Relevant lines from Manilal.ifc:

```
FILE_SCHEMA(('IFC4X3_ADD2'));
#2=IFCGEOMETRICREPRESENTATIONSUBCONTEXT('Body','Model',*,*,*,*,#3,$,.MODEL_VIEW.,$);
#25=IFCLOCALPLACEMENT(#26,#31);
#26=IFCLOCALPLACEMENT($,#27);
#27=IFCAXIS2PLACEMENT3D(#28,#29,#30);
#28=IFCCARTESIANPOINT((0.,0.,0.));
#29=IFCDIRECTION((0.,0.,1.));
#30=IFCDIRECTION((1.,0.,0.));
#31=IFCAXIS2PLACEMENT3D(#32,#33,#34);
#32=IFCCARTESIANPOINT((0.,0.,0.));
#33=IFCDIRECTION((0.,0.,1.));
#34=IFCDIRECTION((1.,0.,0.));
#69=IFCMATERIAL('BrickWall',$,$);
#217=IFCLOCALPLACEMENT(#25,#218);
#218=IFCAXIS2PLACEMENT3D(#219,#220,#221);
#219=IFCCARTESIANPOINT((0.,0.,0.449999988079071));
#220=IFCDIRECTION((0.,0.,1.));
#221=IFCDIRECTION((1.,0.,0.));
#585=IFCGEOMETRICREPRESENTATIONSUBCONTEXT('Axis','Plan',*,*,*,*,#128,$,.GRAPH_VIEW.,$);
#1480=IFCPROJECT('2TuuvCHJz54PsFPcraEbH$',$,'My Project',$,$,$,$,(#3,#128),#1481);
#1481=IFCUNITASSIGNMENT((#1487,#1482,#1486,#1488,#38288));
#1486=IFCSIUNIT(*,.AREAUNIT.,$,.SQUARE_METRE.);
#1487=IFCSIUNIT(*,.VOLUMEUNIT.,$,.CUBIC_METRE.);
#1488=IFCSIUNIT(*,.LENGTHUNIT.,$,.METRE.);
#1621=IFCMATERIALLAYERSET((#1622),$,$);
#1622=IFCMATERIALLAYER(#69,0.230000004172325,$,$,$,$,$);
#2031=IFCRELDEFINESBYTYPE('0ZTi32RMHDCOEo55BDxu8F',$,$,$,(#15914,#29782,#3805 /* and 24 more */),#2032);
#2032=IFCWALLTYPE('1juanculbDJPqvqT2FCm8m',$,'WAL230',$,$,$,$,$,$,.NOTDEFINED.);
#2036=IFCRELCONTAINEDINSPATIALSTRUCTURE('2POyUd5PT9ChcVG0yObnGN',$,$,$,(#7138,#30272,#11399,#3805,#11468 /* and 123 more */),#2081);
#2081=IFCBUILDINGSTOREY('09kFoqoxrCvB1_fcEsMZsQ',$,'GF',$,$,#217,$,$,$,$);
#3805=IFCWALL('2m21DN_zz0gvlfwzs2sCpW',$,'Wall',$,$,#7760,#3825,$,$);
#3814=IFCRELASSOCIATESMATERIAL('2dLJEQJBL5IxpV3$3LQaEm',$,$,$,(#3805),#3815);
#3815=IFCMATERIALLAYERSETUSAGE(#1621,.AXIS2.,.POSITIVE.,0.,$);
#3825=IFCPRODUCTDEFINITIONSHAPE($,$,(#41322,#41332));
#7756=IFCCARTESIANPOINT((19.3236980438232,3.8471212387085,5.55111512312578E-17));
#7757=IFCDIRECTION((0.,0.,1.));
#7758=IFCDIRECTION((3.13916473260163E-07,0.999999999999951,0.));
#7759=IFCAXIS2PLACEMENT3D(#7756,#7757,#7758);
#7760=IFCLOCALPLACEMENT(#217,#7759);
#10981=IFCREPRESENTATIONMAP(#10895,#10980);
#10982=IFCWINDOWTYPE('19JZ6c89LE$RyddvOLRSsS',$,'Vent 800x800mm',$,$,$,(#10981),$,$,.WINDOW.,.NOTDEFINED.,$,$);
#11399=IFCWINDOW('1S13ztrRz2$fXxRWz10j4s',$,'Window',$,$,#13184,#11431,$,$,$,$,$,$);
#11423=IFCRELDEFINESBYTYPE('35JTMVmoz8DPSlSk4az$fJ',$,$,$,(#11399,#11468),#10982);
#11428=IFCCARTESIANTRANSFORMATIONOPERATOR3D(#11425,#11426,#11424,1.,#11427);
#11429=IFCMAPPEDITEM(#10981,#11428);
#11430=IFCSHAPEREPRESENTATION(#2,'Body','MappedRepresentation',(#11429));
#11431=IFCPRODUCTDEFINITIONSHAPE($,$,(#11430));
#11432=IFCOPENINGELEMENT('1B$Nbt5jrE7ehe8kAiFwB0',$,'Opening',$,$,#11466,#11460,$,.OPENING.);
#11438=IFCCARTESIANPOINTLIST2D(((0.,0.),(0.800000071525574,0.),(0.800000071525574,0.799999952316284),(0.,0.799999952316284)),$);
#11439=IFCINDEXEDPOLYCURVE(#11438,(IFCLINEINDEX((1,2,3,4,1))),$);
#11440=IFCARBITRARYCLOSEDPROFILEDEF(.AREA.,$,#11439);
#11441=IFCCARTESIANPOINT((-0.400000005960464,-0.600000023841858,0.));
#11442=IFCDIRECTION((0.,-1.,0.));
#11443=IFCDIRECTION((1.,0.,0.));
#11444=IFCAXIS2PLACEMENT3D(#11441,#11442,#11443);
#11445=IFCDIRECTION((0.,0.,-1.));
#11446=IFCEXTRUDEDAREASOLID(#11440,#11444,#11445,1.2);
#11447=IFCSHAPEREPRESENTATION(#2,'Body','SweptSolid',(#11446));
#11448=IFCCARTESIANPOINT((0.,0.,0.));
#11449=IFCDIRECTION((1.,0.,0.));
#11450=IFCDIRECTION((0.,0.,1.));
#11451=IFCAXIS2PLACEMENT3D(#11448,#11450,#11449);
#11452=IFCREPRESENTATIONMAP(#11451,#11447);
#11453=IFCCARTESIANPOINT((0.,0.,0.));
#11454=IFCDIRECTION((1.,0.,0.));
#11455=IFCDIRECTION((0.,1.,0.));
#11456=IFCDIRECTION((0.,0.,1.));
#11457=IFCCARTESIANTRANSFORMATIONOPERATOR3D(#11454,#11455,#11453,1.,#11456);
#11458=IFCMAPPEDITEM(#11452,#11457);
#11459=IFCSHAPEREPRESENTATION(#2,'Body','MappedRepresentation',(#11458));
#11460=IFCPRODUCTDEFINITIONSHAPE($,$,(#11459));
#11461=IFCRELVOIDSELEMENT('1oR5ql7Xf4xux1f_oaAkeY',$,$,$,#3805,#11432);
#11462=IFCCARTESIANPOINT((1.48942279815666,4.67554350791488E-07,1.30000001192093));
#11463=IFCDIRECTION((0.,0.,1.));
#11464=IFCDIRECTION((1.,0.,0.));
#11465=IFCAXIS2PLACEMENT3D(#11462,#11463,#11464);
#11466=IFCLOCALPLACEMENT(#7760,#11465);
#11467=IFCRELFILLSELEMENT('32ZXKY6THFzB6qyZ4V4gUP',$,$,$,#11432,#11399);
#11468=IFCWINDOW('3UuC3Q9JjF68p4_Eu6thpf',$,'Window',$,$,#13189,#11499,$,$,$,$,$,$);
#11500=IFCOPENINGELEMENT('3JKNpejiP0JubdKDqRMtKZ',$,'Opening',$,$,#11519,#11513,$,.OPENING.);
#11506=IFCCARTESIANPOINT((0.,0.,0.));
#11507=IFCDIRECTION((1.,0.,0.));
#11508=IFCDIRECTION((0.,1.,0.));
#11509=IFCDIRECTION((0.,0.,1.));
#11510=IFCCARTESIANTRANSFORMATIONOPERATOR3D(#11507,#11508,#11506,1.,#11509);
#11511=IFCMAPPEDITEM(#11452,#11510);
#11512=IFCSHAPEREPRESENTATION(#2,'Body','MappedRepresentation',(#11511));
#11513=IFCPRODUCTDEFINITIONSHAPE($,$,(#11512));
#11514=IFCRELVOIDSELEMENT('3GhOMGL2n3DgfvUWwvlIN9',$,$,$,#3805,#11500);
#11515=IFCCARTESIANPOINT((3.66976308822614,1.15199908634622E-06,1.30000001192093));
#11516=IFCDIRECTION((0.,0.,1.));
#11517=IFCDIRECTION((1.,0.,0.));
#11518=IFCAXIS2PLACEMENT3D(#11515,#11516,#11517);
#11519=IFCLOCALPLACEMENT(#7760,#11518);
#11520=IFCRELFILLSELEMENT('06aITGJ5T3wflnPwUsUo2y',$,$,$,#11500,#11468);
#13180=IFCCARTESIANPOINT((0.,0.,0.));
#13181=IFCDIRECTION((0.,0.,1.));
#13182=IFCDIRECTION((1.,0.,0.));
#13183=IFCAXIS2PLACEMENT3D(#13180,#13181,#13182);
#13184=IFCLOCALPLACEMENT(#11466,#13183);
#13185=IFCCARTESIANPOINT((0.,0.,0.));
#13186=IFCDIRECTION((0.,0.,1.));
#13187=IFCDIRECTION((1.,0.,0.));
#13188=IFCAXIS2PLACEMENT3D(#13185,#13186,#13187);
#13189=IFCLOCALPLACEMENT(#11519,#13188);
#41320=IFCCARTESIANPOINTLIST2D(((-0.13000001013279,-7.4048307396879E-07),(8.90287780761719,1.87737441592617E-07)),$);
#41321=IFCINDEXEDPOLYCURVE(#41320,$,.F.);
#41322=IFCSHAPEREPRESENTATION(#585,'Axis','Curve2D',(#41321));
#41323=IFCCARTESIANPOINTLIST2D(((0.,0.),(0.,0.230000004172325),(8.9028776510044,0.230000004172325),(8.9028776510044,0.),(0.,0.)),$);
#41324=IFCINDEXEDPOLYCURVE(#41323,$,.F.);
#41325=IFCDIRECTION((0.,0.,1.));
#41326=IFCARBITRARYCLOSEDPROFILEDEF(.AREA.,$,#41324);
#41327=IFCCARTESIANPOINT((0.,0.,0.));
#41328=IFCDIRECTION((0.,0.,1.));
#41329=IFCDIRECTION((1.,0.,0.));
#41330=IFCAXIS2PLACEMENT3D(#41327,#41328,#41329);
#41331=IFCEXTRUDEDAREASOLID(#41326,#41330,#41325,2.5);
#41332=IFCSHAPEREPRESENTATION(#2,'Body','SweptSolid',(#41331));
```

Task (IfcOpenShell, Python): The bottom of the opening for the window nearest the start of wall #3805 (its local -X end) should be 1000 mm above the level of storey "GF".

```python
import numpy as np
import ifcopenshell
import ifcopenshell.api.geometry
import ifcopenshell.geom
import ifcopenshell.util.element
import ifcopenshell.util.placement
import ifcopenshell.util.shape
import ifcopenshell.util.unit

model = ifcopenshell.open("Manilal.ifc")
unit_scale = ifcopenshell.util.unit.calculate_unit_scale(model)

window = model.by_guid("1S13ztrRz2$fXxRWz10j4s")
opening = window.FillsVoids[0].RelatingOpeningElement
storey = ifcopenshell.util.element.get_container(window, ifc_class="IfcBuildingStorey")
level = ifcopenshell.util.placement.get_local_placement(storey.ObjectPlacement)[2, 3]

# The opening's origin need not be at the sill, so measure its lowest point.
shape = ifcopenshell.geom.create_shape(ifcopenshell.geom.settings(), opening)
bottom = ifcopenshell.util.shape.get_shape_bottom_elevation(shape, shape.geometry) / unit_scale
dz = level + 1.0 - bottom

shift = np.array([0.0, 0.0, dz])
# The window is placed relative to its opening, so it follows when the opening moves.
matrix = ifcopenshell.util.placement.get_local_placement(opening.ObjectPlacement)
matrix[:3, 3] += shift
ifcopenshell.api.geometry.edit_object_placement(
    model, product=opening, matrix=matrix, is_si=False, should_transform_children=True
)

print(f"moved by {dz * unit_scale:+.3f} m")

model.write("Manilal_rev.ifc")
```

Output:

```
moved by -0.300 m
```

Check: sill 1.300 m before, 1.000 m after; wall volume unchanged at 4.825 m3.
